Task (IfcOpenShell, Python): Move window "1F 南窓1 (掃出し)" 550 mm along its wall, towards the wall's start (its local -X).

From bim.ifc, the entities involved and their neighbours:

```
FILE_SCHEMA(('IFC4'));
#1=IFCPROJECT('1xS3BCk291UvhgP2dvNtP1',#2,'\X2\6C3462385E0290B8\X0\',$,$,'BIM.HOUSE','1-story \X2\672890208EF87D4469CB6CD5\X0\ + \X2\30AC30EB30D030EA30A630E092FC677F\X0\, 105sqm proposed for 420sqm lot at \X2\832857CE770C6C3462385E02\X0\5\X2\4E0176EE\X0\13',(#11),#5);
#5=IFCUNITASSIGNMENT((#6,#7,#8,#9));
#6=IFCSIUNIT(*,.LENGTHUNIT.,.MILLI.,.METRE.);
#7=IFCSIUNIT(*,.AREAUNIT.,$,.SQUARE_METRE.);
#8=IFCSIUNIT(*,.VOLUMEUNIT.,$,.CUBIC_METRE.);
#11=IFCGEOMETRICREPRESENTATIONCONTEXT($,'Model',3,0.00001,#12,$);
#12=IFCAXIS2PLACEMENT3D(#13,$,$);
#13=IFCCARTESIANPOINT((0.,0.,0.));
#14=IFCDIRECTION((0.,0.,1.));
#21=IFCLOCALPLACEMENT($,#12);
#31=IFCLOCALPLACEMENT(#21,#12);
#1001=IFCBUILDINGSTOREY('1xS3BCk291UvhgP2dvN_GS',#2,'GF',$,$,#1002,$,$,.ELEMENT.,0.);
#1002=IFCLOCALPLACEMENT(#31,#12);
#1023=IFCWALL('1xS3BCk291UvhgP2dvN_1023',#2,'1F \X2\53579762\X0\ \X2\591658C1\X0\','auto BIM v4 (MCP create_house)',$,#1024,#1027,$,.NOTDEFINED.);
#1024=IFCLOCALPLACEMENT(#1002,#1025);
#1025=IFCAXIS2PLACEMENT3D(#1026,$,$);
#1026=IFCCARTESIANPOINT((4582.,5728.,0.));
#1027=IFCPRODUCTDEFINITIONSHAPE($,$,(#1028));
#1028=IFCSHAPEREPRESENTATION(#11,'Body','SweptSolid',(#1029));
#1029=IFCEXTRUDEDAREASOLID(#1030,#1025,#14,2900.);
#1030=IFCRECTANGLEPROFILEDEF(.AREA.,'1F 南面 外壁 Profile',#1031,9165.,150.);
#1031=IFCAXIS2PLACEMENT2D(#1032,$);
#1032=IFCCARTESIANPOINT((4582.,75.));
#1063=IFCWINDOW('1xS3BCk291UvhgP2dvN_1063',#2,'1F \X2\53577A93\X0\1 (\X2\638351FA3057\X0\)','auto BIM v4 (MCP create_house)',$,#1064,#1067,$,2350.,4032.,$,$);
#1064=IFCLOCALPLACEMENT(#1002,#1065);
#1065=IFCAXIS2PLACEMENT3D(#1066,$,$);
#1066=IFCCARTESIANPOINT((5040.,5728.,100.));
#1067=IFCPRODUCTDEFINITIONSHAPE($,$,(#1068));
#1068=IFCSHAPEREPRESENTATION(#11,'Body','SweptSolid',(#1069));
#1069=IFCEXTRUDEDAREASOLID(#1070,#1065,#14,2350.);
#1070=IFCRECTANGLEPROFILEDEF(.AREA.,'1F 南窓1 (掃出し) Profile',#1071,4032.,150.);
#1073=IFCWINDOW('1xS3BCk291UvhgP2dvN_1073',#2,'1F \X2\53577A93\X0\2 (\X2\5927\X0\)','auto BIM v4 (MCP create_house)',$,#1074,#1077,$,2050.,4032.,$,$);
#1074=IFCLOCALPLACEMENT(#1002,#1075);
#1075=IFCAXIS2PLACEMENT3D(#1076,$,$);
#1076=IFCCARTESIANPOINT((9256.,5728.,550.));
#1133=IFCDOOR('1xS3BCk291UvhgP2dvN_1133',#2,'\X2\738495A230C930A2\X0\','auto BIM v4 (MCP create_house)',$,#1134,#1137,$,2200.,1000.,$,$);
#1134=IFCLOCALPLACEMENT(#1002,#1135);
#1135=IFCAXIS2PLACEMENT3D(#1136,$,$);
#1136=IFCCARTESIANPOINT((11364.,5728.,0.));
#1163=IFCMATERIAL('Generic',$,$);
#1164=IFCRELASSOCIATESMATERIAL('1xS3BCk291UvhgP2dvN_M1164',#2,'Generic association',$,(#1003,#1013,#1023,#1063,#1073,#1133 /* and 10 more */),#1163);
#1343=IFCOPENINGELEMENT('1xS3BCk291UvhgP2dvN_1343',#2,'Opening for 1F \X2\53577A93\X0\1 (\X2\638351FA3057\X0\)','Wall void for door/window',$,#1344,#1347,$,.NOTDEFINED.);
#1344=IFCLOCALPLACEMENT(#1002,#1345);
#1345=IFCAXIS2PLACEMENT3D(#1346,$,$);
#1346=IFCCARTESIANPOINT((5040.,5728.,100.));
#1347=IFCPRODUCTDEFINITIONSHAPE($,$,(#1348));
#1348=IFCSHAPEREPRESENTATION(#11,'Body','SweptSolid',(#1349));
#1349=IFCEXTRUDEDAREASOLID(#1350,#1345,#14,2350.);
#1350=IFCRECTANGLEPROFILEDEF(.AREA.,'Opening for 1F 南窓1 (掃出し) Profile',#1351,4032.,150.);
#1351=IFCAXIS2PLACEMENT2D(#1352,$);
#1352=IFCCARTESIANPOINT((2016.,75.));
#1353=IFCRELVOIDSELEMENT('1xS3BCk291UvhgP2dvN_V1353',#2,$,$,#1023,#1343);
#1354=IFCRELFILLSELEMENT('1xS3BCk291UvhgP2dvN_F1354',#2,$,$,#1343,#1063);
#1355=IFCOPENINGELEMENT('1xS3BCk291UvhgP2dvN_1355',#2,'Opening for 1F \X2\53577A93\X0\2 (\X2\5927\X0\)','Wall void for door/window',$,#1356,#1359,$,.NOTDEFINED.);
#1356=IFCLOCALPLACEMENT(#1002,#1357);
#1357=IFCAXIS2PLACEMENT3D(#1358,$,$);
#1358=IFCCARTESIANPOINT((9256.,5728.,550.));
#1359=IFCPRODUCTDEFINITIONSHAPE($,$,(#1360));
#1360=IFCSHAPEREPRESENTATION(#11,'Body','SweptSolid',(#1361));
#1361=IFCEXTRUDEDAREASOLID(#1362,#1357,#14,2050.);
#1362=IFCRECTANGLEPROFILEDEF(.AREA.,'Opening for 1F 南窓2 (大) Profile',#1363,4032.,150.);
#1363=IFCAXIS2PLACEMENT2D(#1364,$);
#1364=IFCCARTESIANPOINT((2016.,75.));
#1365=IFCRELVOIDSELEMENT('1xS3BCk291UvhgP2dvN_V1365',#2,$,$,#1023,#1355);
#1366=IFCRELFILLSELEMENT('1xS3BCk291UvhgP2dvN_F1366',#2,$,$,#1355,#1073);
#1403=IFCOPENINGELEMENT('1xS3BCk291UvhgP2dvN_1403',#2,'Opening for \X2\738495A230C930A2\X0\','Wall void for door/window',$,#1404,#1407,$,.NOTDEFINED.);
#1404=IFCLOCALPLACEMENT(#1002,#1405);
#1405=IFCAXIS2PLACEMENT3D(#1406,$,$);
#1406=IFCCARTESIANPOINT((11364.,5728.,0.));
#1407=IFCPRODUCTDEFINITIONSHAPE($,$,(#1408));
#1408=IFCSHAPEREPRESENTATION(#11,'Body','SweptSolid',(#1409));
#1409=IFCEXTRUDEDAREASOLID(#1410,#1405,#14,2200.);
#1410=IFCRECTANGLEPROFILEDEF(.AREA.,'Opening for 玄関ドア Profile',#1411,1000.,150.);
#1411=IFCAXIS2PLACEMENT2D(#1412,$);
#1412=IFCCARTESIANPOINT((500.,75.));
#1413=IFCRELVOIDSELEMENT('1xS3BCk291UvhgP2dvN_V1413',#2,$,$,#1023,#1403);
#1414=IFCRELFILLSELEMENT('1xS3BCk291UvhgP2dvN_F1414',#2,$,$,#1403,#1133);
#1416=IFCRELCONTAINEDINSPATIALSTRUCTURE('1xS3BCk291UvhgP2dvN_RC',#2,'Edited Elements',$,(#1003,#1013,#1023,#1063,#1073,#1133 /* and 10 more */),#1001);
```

```python
import ifcopenshell
import ifcopenshell.api.geometry
import ifcopenshell.util.placement
import ifcopenshell.util.unit

model = ifcopenshell.open("bim.ifc")
unit_scale = ifcopenshell.util.unit.calculate_unit_scale(model)

window = model.by_guid("1xS3BCk291UvhgP2dvN_1063")
opening = window.FillsVoids[0].RelatingOpeningElement
wall = opening.VoidsElements[0].RelatingBuildingElement

wall_matrix = ifcopenshell.util.placement.get_local_placement(wall.ObjectPlacement)
shift = wall_matrix[:3, 0] * -0.55 / unit_scale
before = ifcopenshell.util.placement.get_local_placement(window.ObjectPlacement)[:3, 3].copy()

# The window is not placed relative to its opening, so move both.
for product in (opening, window):
    matrix = ifcopenshell.util.placement.get_local_placement(product.ObjectPlacement)
    matrix[:3, 3] += shift
    ifcopenshell.api.geometry.edit_object_placement(model, product=product, matrix=matrix, is_si=False)

after = ifcopenshell.util.placement.get_local_placement(window.ObjectPlacement)[:3, 3]
print("window moved by", (after - before).round(3) + 0.0)

model.write("bim_updated.ifc")
```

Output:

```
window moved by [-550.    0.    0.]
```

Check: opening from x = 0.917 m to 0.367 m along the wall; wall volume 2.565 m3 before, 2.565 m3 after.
